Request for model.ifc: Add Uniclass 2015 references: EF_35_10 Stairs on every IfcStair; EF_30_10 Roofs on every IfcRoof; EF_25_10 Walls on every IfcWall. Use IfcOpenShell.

First a look at what the model holds.

```python
import ifcopenshell

model = ifcopenshell.open("model.ifc")
print(model.schema)
print("classifications:", [c.Name for c in model.by_type("IfcClassification")])
for ifc_class in ("IfcDoor", "IfcRoof", "IfcStair", "IfcWall", "IfcWindow"):
    print(ifc_class, len(model.by_type(ifc_class)))
```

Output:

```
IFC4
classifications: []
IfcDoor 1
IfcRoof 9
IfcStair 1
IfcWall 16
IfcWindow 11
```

```python
import ifcopenshell
import ifcopenshell.api.classification

model = ifcopenshell.open("model.ifc")

system = ifcopenshell.api.classification.add_classification(model, classification="Uniclass 2015")

codes = {
    "IfcStair": ("EF_35_10", "Stairs"),
    "IfcRoof": ("EF_30_10", "Roofs"),
    "IfcWall": ("EF_25_10", "Walls"),
}
for ifc_class, (code, name) in codes.items():
    products = model.by_type(ifc_class)
    ifcopenshell.api.classification.add_reference(
        model, products=products, classification=system, identification=code, name=name
    )
    print(code, len(products))

model.write("model-out.ifc")
```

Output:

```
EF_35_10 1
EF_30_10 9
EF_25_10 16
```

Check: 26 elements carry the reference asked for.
